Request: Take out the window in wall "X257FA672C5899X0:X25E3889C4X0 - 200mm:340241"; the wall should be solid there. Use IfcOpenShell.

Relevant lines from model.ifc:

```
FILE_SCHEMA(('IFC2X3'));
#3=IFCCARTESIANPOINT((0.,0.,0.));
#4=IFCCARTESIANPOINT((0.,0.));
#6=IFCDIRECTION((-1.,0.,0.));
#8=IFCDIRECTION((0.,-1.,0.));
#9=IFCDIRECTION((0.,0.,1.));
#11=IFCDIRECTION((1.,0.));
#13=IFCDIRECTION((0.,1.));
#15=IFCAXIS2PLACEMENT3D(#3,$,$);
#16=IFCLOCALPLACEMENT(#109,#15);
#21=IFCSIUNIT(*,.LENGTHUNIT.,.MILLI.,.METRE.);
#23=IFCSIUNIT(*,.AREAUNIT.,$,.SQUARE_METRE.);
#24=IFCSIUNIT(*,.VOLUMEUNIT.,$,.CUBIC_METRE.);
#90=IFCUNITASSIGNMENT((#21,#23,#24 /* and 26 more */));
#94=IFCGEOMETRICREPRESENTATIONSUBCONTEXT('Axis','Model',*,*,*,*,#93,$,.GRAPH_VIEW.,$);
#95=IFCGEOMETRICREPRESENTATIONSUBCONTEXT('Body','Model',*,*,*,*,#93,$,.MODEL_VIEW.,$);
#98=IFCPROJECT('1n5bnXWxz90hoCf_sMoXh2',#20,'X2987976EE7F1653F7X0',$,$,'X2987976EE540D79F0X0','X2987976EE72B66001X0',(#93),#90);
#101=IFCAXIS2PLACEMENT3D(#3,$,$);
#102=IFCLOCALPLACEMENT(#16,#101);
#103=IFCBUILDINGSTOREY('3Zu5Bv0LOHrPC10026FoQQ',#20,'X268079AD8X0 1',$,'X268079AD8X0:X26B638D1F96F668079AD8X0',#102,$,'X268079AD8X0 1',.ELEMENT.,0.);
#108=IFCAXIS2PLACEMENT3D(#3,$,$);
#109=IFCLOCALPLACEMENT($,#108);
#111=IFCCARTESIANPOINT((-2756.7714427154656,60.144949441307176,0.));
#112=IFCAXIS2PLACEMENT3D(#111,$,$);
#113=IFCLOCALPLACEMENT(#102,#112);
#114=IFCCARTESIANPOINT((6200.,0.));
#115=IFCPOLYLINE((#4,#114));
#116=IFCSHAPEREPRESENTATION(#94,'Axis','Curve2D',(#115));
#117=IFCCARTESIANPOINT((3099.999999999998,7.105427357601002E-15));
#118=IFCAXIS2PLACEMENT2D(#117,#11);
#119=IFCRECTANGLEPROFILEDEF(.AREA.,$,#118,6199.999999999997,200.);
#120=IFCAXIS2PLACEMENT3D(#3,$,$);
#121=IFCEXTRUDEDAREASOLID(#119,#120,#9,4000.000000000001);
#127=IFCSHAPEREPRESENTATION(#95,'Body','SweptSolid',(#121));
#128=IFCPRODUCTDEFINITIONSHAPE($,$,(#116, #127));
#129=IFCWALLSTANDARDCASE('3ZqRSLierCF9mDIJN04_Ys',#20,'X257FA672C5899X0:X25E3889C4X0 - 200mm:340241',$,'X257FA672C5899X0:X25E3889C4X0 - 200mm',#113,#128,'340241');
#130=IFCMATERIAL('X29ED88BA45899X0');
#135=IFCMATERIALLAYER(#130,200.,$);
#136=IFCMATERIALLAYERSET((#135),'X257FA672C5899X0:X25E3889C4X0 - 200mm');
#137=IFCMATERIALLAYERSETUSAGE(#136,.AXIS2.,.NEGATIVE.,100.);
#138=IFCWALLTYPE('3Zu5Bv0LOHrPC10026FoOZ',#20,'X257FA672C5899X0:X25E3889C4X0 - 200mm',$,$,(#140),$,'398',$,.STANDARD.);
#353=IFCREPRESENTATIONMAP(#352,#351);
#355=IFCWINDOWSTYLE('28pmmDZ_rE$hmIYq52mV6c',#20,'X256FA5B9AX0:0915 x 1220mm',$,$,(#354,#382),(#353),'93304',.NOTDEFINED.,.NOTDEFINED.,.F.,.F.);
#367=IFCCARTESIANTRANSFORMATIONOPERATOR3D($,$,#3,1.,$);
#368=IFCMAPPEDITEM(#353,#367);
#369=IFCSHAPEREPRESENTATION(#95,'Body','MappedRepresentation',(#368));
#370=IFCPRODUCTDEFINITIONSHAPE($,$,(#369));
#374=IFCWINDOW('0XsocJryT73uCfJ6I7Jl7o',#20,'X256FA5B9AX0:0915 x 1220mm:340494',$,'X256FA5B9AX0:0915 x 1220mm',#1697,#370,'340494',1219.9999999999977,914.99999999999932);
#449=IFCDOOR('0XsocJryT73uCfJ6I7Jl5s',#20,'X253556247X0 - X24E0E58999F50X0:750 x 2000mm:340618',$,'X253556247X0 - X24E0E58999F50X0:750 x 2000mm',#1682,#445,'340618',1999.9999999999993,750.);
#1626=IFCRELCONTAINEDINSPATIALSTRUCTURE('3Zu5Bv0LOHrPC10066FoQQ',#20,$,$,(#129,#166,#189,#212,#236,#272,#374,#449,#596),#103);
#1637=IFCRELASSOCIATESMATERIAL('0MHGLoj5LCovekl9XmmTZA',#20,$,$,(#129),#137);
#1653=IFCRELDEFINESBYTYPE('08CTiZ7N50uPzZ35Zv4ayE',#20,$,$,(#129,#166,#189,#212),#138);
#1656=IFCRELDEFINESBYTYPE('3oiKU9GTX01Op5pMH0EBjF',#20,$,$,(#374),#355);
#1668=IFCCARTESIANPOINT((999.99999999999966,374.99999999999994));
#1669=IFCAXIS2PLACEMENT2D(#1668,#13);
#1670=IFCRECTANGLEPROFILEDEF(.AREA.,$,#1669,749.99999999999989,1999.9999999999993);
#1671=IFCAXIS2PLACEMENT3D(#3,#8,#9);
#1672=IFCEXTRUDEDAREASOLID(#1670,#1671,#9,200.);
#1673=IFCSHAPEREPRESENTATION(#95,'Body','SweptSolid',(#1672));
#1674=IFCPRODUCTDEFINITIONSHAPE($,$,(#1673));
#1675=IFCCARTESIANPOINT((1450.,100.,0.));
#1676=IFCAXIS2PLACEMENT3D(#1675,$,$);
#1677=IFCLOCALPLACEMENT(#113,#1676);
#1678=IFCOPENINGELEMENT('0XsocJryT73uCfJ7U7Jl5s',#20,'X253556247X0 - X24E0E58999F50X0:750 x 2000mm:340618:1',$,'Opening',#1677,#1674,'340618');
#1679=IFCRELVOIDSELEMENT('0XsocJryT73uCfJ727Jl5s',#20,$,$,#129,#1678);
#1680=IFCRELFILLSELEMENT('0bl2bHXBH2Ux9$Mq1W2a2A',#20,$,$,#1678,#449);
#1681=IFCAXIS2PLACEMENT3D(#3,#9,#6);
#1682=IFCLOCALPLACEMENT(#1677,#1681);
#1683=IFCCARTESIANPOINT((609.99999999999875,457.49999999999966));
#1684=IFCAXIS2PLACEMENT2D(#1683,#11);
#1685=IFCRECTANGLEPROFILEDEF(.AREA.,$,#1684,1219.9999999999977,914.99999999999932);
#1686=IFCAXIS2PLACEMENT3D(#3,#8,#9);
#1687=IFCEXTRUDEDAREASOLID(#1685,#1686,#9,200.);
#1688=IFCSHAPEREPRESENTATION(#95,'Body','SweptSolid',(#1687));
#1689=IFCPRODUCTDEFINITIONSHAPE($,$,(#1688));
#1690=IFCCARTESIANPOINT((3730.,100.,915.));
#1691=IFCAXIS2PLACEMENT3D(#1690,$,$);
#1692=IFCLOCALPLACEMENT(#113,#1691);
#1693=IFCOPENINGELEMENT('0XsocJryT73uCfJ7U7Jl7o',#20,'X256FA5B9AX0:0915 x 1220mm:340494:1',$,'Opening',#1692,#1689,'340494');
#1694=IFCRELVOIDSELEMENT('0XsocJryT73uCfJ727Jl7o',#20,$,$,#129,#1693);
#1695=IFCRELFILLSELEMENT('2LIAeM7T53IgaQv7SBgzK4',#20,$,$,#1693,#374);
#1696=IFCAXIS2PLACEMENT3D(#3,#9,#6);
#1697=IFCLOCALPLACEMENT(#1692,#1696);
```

```python
import ifcopenshell
import ifcopenshell.api.feature
import ifcopenshell.api.root
import ifcopenshell.geom
import ifcopenshell.util.shape

model = ifcopenshell.open("model.ifc")
settings = ifcopenshell.geom.settings()


def volume(element):
    """Net volume in cubic metres, openings subtracted."""
    shape = ifcopenshell.geom.create_shape(settings, element)
    return ifcopenshell.util.shape.get_volume(shape.geometry)


window = model.by_guid("0XsocJryT73uCfJ6I7Jl7o")
opening = window.FillsVoids[0].RelatingOpeningElement
wall = opening.VoidsElements[0].RelatingBuildingElement
before = volume(wall)

ifcopenshell.api.root.remove_product(model, product=window)
ifcopenshell.api.feature.remove_feature(model, feature=opening)

after = volume(wall)

print(f"wall volume {before:.3f} -> {after:.3f} m3")

model.write("model_rev.ifc")
```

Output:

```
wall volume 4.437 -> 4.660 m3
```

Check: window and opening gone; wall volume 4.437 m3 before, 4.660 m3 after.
